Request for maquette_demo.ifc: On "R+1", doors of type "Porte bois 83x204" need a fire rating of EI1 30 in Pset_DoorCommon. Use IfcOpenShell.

First a look at what the model holds.

```python
import ifcopenshell
import ifcopenshell.util.element

model = ifcopenshell.open("maquette_demo.ifc")
print(model.schema)
storey = next(s for s in model.by_type("IfcBuildingStorey") if s.Name == "R+1")
doors = [e for e in ifcopenshell.util.element.get_decomposition(storey) if e.is_a("IfcDoor")]
seen = {}
for e in doors:
    element_type = ifcopenshell.util.element.get_type(e)
    key = (element_type.Name if element_type != e and element_type else None, ifcopenshell.util.element.get_pset(e, "Pset_DoorCommon", "FireRating"))
    seen[key] = seen.get(key, 0) + 1
for (name, value), count in sorted(seen.items(), key=str):
    print(count, "x", name, "|", value)
```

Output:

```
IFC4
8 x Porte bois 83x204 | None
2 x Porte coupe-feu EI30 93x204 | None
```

```python
import ifcopenshell
import ifcopenshell.api.pset
import ifcopenshell.util.element

model = ifcopenshell.open("maquette_demo.ifc")

storey = next(s for s in model.by_type("IfcBuildingStorey") if s.Name == "R+1")
doors = [e for e in ifcopenshell.util.element.get_decomposition(storey) if e.is_a("IfcDoor")]

count = 0
for e in doors:
    element_type = ifcopenshell.util.element.get_type(e)
    if element_type in (None, e) or element_type.Name != "Porte bois 83x204":
        continue
    # add_pset returns the element's existing set when there is one.
    pset = ifcopenshell.api.pset.add_pset(model, product=e, name="Pset_DoorCommon")
    ifcopenshell.api.pset.edit_pset(model, pset=pset, properties={"FireRating": "EI1 30"})
    count += 1

print(count, "doors updated")

model.write("maquette_demo_rev.ifc")
```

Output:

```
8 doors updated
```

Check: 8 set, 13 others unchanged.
